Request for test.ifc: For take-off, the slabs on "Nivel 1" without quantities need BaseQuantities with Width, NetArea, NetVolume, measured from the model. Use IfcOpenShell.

First a look at what the model holds.

```python
import ifcopenshell
import ifcopenshell.util.element
import ifcopenshell.util.unit

model = ifcopenshell.open("test.ifc")
print(model.schema)
for unit_type in ("LENGTHUNIT", "AREAUNIT", "VOLUMEUNIT"):
    print(unit_type, ifcopenshell.util.unit.calculate_unit_scale(model, unit_type))
storey = next(s for s in model.by_type("IfcBuildingStorey") if s.Name == "Nivel 1")
slabs = [e for e in ifcopenshell.util.element.get_decomposition(storey) if e.is_a("IfcSlab")]
for e in sorted(slabs, key=lambda e: e.id()):
    print(e.id(), e.is_a(), e.Name, list(ifcopenshell.util.element.get_psets(e, qtos_only=True)), sep=" | ")
```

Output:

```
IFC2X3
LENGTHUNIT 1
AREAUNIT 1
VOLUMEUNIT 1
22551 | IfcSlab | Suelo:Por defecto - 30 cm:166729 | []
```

```python
import ifcopenshell
import ifcopenshell.api.pset
import ifcopenshell.geom
import ifcopenshell.util.element
import ifcopenshell.util.shape
import ifcopenshell.util.unit

model = ifcopenshell.open("test.ifc")
unit_scale = ifcopenshell.util.unit.calculate_unit_scale(model)
area_scale = ifcopenshell.util.unit.calculate_unit_scale(model, "AREAUNIT")
volume_scale = ifcopenshell.util.unit.calculate_unit_scale(model, "VOLUMEUNIT")
settings = ifcopenshell.geom.settings()

storey = next(s for s in model.by_type("IfcBuildingStorey") if s.Name == "Nivel 1")
slabs = [e for e in ifcopenshell.util.element.get_decomposition(storey) if e.is_a("IfcSlab")]

for e in sorted(slabs, key=lambda e: e.id()):
    if ifcopenshell.util.element.get_psets(e, qtos_only=True, should_inherit=False):
        continue
    # Geometry comes back in metres, in the element's own axes.
    shape = ifcopenshell.geom.create_shape(settings, e)
    values = {
        "Width": ifcopenshell.util.shape.get_z(shape.geometry) / unit_scale,
        "NetArea": ifcopenshell.util.shape.get_footprint_area(shape.geometry) / area_scale,
        "NetVolume": ifcopenshell.util.shape.get_volume(shape.geometry) / volume_scale,
    }
    qto = ifcopenshell.api.pset.add_qto(model, product=e, name="BaseQuantities")
    ifcopenshell.api.pset.edit_qto(model, qto=qto, properties=values)
    print(e.id(), {k: round(v, 3) for k, v in values.items()})

model.write("test-out.ifc")
```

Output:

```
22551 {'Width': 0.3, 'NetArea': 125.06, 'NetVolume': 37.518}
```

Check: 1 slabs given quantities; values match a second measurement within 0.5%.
